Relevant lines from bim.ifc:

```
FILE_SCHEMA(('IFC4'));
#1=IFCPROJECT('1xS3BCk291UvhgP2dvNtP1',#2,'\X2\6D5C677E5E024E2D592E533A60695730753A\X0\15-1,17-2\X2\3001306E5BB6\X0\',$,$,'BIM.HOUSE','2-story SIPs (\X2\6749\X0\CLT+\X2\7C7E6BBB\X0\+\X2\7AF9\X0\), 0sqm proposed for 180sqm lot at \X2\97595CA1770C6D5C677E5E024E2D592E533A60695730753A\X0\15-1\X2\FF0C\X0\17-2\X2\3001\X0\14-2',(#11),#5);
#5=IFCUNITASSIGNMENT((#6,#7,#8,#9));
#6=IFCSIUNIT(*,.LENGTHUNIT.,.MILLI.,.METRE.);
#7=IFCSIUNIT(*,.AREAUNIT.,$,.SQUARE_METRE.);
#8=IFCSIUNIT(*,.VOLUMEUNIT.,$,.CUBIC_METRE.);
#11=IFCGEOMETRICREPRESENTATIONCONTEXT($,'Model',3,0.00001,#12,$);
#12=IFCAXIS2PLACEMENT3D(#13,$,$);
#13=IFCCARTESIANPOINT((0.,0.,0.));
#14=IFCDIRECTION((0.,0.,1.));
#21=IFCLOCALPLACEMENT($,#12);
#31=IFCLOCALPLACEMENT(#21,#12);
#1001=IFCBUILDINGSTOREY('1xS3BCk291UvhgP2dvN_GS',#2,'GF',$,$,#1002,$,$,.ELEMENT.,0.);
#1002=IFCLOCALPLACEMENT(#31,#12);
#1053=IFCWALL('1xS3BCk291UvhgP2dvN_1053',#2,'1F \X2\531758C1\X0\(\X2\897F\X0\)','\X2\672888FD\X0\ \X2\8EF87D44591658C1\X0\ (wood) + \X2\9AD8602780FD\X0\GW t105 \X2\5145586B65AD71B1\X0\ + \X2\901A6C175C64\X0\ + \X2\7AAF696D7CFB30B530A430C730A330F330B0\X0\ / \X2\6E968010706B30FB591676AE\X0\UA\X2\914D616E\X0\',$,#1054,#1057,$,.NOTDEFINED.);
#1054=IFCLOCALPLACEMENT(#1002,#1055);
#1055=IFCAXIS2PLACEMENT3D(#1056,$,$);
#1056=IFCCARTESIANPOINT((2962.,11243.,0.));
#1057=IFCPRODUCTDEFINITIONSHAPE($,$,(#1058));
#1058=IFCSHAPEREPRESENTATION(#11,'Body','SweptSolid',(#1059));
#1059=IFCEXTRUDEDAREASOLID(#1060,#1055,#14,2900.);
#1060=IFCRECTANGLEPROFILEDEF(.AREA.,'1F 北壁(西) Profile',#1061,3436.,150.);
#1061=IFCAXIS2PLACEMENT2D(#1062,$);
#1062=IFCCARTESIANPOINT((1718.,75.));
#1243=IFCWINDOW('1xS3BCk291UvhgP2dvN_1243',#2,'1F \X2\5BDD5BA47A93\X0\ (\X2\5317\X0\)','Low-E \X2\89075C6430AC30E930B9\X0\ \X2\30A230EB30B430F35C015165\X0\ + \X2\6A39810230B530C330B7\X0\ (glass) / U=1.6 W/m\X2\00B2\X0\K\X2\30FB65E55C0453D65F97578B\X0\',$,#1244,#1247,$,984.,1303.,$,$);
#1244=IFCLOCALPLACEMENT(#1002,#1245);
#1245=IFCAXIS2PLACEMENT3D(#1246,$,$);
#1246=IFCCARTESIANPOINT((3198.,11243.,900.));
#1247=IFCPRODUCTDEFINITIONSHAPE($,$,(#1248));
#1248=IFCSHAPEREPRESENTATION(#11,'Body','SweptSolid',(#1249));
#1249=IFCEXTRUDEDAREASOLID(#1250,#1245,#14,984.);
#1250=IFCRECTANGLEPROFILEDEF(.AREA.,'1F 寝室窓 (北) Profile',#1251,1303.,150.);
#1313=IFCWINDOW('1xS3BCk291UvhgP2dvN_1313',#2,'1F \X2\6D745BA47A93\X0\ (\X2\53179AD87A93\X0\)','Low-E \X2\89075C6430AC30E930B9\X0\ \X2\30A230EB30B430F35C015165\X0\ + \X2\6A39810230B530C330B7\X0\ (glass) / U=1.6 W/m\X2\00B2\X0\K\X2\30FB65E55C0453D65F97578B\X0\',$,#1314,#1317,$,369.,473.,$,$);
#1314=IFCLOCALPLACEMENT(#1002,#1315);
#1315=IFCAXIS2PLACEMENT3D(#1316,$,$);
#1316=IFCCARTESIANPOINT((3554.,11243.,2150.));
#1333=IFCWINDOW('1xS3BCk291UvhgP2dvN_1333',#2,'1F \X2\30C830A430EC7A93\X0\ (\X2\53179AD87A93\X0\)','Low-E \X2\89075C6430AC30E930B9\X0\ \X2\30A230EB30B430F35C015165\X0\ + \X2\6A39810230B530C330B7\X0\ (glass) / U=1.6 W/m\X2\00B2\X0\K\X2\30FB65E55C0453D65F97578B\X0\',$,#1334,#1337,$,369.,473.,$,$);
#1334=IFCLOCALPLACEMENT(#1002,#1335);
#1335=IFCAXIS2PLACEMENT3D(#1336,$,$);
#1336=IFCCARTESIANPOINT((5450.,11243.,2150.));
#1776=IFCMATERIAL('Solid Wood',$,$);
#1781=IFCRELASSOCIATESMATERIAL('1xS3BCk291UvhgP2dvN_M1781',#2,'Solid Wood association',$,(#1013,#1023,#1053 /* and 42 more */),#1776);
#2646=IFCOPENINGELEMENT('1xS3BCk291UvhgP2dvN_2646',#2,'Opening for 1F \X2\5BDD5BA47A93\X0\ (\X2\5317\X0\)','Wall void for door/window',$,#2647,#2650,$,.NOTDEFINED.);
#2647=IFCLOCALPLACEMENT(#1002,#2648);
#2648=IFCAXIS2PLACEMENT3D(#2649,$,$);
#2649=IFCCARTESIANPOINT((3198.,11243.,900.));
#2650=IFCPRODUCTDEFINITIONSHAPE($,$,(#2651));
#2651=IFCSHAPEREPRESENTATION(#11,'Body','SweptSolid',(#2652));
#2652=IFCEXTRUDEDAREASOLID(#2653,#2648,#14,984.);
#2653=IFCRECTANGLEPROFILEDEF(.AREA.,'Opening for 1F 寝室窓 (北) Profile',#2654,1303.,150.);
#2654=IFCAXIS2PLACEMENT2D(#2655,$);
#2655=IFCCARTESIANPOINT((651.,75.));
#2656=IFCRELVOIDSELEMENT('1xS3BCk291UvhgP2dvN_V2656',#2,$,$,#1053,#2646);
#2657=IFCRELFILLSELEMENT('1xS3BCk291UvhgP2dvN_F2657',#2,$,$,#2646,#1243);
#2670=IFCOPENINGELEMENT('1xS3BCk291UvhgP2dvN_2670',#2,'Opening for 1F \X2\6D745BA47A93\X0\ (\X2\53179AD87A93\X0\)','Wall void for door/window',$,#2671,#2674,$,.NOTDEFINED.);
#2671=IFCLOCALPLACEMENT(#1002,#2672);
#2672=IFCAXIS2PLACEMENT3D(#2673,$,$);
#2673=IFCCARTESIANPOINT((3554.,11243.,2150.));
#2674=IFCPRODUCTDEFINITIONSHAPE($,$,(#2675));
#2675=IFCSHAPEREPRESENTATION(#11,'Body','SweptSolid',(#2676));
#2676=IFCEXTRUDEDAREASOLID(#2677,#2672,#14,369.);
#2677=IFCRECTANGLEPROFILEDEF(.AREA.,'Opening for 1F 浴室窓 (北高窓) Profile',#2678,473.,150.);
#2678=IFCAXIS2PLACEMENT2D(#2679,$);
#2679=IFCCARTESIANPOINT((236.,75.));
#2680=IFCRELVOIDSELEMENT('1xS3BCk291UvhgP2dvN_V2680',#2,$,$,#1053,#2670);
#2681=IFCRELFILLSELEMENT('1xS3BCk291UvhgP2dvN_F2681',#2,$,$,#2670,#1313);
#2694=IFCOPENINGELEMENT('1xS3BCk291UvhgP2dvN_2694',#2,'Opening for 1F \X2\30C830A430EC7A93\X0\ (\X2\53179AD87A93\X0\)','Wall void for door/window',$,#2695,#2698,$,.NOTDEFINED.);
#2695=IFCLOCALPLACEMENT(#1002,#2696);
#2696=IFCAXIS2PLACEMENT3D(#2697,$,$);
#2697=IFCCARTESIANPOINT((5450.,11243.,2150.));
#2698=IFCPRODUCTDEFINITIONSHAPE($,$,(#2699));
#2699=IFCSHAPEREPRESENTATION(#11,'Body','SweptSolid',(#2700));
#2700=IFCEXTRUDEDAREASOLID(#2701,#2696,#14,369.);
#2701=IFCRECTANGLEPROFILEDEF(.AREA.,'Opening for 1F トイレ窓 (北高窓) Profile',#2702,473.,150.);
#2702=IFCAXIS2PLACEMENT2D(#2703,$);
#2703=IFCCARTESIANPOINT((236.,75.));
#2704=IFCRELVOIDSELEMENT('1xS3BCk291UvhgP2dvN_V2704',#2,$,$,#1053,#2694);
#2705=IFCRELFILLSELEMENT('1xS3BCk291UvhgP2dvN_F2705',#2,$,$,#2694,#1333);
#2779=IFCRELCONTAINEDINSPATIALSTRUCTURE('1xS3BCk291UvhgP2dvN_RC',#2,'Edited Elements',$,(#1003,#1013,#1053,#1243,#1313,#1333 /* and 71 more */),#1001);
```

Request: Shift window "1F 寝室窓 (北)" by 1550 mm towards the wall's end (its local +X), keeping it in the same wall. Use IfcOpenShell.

```python
import ifcopenshell
import ifcopenshell.api.geometry
import ifcopenshell.util.placement
import ifcopenshell.util.unit

model = ifcopenshell.open("bim.ifc")
unit_scale = ifcopenshell.util.unit.calculate_unit_scale(model)

window = model.by_guid("1xS3BCk291UvhgP2dvN_1243")
opening = window.FillsVoids[0].RelatingOpeningElement
wall = opening.VoidsElements[0].RelatingBuildingElement

wall_matrix = ifcopenshell.util.placement.get_local_placement(wall.ObjectPlacement)
shift = wall_matrix[:3, 0] * 1.55 / unit_scale
before = ifcopenshell.util.placement.get_local_placement(window.ObjectPlacement)[:3, 3].copy()

# The window is not placed relative to its opening, so move both.
for product in (opening, window):
    matrix = ifcopenshell.util.placement.get_local_placement(product.ObjectPlacement)
    matrix[:3, 3] += shift
    ifcopenshell.api.geometry.edit_object_placement(model, product=product, matrix=matrix, is_si=False)

after = ifcopenshell.util.placement.get_local_placement(window.ObjectPlacement)[:3, 3]
print("window moved by", (after - before).round(3) + 0.0)

model.write("bim_updated.ifc")
```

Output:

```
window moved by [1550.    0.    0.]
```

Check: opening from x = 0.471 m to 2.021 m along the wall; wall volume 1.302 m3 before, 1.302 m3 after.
